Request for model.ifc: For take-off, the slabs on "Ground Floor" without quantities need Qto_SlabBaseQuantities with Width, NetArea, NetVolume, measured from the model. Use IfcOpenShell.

First a look at what the model holds.

```python
import ifcopenshell
import ifcopenshell.util.element
import ifcopenshell.util.unit

model = ifcopenshell.open("model.ifc")
print(model.schema)
for unit_type in ("LENGTHUNIT", "AREAUNIT", "VOLUMEUNIT"):
    print(unit_type, ifcopenshell.util.unit.calculate_unit_scale(model, unit_type))
storey = next(s for s in model.by_type("IfcBuildingStorey") if s.Name == "Ground Floor")
slabs = [e for e in ifcopenshell.util.element.get_decomposition(storey) if e.is_a("IfcSlab")]
for e in sorted(slabs, key=lambda e: e.id()):
    print(e.id(), e.is_a(), e.Name, list(ifcopenshell.util.element.get_psets(e, qtos_only=True)), sep=" | ")
```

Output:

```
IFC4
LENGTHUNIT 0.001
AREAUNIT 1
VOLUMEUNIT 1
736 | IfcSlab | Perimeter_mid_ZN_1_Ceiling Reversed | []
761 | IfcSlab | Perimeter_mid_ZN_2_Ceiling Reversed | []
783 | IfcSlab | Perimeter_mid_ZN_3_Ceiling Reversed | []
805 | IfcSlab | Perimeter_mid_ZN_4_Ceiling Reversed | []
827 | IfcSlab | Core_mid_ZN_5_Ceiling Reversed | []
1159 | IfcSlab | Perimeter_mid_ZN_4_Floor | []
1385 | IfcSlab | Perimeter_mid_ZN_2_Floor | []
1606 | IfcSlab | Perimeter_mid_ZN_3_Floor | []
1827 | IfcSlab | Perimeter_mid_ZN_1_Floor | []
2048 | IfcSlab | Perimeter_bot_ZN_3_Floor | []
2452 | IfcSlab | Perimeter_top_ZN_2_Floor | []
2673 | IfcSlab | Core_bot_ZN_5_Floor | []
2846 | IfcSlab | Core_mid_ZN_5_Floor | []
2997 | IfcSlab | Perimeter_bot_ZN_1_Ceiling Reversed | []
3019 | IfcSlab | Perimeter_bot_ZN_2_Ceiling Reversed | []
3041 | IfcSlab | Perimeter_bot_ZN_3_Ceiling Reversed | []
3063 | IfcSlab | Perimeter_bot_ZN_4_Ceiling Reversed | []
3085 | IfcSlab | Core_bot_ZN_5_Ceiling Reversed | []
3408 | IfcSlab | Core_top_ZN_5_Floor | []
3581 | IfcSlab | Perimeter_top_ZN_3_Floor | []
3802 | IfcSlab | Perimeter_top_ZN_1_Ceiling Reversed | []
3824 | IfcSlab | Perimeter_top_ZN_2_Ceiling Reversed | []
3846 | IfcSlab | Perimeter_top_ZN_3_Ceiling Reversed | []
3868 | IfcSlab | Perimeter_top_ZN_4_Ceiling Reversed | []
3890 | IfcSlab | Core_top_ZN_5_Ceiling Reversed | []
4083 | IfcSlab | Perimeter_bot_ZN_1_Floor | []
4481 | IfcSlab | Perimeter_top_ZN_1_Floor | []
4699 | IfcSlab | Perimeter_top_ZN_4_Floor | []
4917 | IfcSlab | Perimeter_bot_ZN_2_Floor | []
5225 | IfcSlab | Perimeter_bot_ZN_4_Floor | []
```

```python
import ifcopenshell
import ifcopenshell.api.pset
import ifcopenshell.geom
import ifcopenshell.util.element
import ifcopenshell.util.shape
import ifcopenshell.util.unit

model = ifcopenshell.open("model.ifc")
unit_scale = ifcopenshell.util.unit.calculate_unit_scale(model)
area_scale = ifcopenshell.util.unit.calculate_unit_scale(model, "AREAUNIT")
volume_scale = ifcopenshell.util.unit.calculate_unit_scale(model, "VOLUMEUNIT")
settings = ifcopenshell.geom.settings()

storey = next(s for s in model.by_type("IfcBuildingStorey") if s.Name == "Ground Floor")
slabs = [e for e in ifcopenshell.util.element.get_decomposition(storey) if e.is_a("IfcSlab")]

for e in sorted(slabs, key=lambda e: e.id()):
    if ifcopenshell.util.element.get_psets(e, qtos_only=True, should_inherit=False):
        continue
    # Geometry comes back in metres, in the element's own axes.
    shape = ifcopenshell.geom.create_shape(settings, e)
    values = {
        "Width": ifcopenshell.util.shape.get_z(shape.geometry) / unit_scale,
        "NetArea": ifcopenshell.util.shape.get_footprint_area(shape.geometry) / area_scale,
        "NetVolume": ifcopenshell.util.shape.get_volume(shape.geometry) / volume_scale,
    }
    qto = ifcopenshell.api.pset.add_qto(model, product=e, name="Qto_SlabBaseQuantities")
    ifcopenshell.api.pset.edit_qto(model, qto=qto, properties=values)
    print(e.id(), {k: round(v, 3) for k, v in values.items()})

model.write("model_edited.ifc")
```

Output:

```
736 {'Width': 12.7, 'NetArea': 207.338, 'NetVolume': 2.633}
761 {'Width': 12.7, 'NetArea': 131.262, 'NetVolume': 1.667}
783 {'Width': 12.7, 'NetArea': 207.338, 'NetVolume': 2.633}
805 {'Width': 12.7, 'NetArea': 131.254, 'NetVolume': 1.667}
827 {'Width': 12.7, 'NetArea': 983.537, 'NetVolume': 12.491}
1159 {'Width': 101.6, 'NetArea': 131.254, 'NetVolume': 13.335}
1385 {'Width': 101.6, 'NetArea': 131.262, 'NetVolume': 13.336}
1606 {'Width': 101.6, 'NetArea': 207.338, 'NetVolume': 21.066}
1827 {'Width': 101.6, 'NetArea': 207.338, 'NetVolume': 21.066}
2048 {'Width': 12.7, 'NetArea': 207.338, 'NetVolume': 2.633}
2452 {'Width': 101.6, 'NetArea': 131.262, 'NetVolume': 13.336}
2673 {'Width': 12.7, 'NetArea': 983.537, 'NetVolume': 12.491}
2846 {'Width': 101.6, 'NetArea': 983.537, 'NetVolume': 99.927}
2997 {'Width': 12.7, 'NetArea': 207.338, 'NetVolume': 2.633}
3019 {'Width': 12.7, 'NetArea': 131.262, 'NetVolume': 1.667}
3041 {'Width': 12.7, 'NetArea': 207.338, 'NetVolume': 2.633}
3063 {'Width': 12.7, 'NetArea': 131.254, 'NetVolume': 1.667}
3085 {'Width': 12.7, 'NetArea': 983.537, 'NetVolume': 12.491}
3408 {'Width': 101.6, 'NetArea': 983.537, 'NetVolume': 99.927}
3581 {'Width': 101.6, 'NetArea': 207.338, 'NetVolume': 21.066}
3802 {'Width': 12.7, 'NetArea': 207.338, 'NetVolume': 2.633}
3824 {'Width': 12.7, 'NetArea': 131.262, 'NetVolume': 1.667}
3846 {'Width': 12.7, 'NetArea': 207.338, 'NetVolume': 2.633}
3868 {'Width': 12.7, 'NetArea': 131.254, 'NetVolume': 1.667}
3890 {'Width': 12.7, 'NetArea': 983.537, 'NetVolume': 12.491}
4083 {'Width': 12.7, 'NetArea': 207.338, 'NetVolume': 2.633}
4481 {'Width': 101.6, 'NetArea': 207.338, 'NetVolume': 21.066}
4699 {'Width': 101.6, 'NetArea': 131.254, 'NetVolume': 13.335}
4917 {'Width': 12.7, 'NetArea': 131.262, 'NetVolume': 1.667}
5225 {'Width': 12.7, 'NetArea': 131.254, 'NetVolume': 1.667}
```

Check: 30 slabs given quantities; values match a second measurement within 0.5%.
